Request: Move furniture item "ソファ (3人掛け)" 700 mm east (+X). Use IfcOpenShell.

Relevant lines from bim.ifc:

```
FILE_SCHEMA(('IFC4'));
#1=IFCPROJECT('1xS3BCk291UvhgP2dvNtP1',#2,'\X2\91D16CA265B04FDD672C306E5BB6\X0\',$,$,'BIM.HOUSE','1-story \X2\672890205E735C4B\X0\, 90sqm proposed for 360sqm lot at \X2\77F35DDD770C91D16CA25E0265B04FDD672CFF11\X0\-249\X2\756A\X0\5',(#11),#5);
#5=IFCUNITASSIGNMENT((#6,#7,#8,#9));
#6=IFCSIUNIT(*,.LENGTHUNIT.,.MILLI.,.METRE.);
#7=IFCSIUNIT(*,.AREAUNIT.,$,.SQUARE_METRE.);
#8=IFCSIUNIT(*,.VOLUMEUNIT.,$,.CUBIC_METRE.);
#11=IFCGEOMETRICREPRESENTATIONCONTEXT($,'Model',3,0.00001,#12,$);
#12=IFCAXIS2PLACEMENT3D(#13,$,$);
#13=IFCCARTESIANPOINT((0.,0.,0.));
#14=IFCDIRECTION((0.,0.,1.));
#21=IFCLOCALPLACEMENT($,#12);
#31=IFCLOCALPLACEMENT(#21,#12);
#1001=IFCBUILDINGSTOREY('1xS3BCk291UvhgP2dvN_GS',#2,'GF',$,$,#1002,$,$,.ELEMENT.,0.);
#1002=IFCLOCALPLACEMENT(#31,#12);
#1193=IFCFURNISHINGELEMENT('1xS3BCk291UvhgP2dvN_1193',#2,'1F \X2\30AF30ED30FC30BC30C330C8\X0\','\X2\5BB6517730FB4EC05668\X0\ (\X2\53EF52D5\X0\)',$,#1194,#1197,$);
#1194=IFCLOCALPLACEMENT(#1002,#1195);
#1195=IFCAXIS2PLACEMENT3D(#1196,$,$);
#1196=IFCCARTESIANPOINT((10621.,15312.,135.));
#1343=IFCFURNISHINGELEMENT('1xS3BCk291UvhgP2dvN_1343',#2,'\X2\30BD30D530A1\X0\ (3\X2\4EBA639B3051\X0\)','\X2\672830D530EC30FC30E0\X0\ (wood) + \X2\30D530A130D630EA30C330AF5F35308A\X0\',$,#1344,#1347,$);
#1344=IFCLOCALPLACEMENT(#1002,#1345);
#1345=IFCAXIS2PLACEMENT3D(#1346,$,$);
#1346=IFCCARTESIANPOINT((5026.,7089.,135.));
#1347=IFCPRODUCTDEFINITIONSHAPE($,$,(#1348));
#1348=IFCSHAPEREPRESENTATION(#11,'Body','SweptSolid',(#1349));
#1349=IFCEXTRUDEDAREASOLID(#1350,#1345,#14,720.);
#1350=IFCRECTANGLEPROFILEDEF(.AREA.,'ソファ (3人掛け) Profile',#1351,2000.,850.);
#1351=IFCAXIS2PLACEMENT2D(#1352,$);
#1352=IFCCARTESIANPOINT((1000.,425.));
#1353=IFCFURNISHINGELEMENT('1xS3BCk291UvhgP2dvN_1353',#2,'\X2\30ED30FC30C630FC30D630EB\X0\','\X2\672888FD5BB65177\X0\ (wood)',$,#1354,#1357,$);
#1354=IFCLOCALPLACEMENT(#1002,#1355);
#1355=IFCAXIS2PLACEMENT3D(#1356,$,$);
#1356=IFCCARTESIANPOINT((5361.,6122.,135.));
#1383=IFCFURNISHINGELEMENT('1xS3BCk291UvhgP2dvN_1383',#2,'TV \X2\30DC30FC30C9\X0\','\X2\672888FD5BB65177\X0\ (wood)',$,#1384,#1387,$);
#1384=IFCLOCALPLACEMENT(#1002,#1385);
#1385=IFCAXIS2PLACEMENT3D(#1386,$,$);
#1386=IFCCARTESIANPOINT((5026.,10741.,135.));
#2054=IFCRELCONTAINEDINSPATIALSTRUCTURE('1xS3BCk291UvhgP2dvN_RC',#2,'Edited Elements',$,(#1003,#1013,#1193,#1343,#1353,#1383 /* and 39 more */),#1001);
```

```python
import ifcopenshell
import ifcopenshell.api.geometry
import ifcopenshell.util.placement

model = ifcopenshell.open("bim.ifc")

item = model.by_id(1343)
matrix = ifcopenshell.util.placement.get_local_placement(item.ObjectPlacement)
matrix[0, 3] += 700.0
ifcopenshell.api.geometry.edit_object_placement(model, product=item, matrix=matrix, is_si=False)

print(ifcopenshell.util.placement.get_local_placement(item.ObjectPlacement).round(3) + 0.0)

model.write("bim-out.ifc")
```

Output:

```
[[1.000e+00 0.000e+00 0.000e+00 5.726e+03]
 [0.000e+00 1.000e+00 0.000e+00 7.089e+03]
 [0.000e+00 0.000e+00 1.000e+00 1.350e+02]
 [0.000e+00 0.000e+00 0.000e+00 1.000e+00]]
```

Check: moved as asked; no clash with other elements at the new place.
